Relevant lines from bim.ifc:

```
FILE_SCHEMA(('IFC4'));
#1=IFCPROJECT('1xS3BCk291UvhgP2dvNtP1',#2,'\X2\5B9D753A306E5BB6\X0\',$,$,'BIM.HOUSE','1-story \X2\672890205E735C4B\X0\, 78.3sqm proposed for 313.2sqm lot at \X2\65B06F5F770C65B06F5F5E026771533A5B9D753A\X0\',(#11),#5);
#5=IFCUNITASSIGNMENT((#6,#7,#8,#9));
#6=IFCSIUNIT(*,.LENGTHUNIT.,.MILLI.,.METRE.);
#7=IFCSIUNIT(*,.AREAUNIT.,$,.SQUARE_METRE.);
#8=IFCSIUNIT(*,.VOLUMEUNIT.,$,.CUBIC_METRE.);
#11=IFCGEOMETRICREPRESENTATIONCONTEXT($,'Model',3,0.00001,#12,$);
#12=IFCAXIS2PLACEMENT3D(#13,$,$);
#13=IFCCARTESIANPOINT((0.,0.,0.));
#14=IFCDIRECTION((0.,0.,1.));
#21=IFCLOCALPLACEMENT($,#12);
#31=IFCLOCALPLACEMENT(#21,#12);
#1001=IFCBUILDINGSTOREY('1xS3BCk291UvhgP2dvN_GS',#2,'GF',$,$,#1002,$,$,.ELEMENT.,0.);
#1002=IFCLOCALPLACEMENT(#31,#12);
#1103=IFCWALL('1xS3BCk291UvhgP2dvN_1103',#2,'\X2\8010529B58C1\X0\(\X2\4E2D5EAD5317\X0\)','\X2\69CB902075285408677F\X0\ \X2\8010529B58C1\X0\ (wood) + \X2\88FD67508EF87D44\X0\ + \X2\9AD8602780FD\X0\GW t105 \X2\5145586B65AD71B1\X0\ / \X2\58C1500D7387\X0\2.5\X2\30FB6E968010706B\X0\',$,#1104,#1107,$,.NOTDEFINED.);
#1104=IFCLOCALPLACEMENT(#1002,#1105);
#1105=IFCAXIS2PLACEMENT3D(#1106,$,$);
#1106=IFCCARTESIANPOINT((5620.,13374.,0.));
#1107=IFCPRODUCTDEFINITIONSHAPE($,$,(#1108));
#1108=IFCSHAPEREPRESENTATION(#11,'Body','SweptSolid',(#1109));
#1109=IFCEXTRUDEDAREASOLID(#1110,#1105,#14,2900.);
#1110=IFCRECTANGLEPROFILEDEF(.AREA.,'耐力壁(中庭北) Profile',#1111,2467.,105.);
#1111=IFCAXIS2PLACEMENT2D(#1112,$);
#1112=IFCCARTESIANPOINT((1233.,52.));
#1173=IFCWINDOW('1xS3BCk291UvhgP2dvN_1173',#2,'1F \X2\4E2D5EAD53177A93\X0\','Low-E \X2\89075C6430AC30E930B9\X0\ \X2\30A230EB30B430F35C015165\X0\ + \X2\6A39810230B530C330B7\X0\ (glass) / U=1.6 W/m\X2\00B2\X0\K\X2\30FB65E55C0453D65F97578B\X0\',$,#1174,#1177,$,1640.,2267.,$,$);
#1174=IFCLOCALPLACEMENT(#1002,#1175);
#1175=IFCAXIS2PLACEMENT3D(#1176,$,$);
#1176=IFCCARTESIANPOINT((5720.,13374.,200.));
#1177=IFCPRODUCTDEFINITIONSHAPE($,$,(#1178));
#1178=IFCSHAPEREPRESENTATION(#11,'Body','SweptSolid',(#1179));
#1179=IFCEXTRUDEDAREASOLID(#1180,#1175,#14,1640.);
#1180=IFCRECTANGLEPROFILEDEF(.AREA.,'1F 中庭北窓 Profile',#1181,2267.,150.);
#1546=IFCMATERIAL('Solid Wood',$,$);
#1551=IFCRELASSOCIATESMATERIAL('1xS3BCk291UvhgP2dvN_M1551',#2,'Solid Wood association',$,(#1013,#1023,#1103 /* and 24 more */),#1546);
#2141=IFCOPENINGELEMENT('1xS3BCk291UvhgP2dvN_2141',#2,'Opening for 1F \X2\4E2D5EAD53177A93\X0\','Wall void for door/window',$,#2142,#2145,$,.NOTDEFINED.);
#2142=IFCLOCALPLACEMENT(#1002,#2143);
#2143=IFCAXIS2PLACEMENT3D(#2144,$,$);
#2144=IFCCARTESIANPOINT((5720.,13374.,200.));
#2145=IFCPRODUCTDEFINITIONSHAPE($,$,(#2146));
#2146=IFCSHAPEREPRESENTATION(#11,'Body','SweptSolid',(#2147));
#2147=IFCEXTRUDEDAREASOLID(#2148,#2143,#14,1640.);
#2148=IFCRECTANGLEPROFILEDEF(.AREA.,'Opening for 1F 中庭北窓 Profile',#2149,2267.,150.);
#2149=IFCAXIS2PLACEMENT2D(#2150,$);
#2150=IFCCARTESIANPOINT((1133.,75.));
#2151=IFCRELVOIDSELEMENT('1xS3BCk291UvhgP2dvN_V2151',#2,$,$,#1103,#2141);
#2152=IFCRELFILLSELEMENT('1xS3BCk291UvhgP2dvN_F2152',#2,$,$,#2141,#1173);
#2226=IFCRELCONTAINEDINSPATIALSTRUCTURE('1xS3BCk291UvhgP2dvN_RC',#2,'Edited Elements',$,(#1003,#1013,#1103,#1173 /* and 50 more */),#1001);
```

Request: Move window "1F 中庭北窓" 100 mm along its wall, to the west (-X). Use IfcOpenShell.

```python
import ifcopenshell
import ifcopenshell.api.geometry
import ifcopenshell.util.placement
import ifcopenshell.util.unit

model = ifcopenshell.open("bim.ifc")
unit_scale = ifcopenshell.util.unit.calculate_unit_scale(model)

window = model.by_guid("1xS3BCk291UvhgP2dvN_1173")
opening = window.FillsVoids[0].RelatingOpeningElement
wall = opening.VoidsElements[0].RelatingBuildingElement

wall_matrix = ifcopenshell.util.placement.get_local_placement(wall.ObjectPlacement)
shift = wall_matrix[:3, 0] * -0.1 / unit_scale
before = ifcopenshell.util.placement.get_local_placement(window.ObjectPlacement)[:3, 3].copy()

# The window is not placed relative to its opening, so move both.
for product in (opening, window):
    matrix = ifcopenshell.util.placement.get_local_placement(product.ObjectPlacement)
    matrix[:3, 3] += shift
    ifcopenshell.api.geometry.edit_object_placement(model, product=product, matrix=matrix, is_si=False)

after = ifcopenshell.util.placement.get_local_placement(window.ObjectPlacement)[:3, 3]
print("window moved by", (after - before).round(3) + 0.0)

model.write("bim-out.ifc")
```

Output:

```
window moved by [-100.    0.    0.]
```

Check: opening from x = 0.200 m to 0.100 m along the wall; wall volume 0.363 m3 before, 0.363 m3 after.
